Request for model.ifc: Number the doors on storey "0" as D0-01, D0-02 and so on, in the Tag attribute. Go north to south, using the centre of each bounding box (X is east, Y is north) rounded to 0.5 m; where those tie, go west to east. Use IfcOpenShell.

First a look at what the model holds.

```python
import ifcopenshell
import ifcopenshell.util.element
import ifcopenshell.util.placement

model = ifcopenshell.open("model.ifc")
print(model.schema)
storey = next(s for s in model.by_type("IfcBuildingStorey") if s.Name == "0")
doors = [e for e in ifcopenshell.util.element.get_decomposition(storey) if e.is_a("IfcDoor")]
for e in sorted(doors, key=lambda e: e.id()):
    origin = ifcopenshell.util.placement.get_local_placement(e.ObjectPlacement)[:3, 3]
    print(e.id(), e.Tag, e.Name, origin.round(2) + 0.0, sep=" | ")
```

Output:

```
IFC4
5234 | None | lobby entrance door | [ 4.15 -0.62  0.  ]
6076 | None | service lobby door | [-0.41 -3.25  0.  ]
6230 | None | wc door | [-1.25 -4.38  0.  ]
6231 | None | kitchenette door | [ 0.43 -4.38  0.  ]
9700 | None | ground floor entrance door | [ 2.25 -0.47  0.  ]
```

```python
import ifcopenshell
import ifcopenshell.geom
import ifcopenshell.util.element
import ifcopenshell.util.shape

model = ifcopenshell.open("model.ifc")
settings = ifcopenshell.geom.settings()
settings.set("use-world-coords", True)


def centre(element):
    shape = ifcopenshell.geom.create_shape(settings, element)
    return ifcopenshell.util.shape.get_bbox_centroid(shape.geometry)


storey = next(s for s in model.by_type("IfcBuildingStorey") if s.Name == "0")
doors = [e for e in ifcopenshell.util.element.get_decomposition(storey) if e.is_a("IfcDoor")]

# Insertion points can sit at a corner or the storey origin, so sort by the geometry (in metres).
centres = {e: centre(e) for e in doors}
doors.sort(key=lambda e: (-round(centres[e][1] / 0.5), centres[e][0]))

for i, e in enumerate(doors, start=1):
    number = f"D0-{i:02d}"
    e.Tag = number
    print(e.id(), number)

model.write("model_rev.ifc")
```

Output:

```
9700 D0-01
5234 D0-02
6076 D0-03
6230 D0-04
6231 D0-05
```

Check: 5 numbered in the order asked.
